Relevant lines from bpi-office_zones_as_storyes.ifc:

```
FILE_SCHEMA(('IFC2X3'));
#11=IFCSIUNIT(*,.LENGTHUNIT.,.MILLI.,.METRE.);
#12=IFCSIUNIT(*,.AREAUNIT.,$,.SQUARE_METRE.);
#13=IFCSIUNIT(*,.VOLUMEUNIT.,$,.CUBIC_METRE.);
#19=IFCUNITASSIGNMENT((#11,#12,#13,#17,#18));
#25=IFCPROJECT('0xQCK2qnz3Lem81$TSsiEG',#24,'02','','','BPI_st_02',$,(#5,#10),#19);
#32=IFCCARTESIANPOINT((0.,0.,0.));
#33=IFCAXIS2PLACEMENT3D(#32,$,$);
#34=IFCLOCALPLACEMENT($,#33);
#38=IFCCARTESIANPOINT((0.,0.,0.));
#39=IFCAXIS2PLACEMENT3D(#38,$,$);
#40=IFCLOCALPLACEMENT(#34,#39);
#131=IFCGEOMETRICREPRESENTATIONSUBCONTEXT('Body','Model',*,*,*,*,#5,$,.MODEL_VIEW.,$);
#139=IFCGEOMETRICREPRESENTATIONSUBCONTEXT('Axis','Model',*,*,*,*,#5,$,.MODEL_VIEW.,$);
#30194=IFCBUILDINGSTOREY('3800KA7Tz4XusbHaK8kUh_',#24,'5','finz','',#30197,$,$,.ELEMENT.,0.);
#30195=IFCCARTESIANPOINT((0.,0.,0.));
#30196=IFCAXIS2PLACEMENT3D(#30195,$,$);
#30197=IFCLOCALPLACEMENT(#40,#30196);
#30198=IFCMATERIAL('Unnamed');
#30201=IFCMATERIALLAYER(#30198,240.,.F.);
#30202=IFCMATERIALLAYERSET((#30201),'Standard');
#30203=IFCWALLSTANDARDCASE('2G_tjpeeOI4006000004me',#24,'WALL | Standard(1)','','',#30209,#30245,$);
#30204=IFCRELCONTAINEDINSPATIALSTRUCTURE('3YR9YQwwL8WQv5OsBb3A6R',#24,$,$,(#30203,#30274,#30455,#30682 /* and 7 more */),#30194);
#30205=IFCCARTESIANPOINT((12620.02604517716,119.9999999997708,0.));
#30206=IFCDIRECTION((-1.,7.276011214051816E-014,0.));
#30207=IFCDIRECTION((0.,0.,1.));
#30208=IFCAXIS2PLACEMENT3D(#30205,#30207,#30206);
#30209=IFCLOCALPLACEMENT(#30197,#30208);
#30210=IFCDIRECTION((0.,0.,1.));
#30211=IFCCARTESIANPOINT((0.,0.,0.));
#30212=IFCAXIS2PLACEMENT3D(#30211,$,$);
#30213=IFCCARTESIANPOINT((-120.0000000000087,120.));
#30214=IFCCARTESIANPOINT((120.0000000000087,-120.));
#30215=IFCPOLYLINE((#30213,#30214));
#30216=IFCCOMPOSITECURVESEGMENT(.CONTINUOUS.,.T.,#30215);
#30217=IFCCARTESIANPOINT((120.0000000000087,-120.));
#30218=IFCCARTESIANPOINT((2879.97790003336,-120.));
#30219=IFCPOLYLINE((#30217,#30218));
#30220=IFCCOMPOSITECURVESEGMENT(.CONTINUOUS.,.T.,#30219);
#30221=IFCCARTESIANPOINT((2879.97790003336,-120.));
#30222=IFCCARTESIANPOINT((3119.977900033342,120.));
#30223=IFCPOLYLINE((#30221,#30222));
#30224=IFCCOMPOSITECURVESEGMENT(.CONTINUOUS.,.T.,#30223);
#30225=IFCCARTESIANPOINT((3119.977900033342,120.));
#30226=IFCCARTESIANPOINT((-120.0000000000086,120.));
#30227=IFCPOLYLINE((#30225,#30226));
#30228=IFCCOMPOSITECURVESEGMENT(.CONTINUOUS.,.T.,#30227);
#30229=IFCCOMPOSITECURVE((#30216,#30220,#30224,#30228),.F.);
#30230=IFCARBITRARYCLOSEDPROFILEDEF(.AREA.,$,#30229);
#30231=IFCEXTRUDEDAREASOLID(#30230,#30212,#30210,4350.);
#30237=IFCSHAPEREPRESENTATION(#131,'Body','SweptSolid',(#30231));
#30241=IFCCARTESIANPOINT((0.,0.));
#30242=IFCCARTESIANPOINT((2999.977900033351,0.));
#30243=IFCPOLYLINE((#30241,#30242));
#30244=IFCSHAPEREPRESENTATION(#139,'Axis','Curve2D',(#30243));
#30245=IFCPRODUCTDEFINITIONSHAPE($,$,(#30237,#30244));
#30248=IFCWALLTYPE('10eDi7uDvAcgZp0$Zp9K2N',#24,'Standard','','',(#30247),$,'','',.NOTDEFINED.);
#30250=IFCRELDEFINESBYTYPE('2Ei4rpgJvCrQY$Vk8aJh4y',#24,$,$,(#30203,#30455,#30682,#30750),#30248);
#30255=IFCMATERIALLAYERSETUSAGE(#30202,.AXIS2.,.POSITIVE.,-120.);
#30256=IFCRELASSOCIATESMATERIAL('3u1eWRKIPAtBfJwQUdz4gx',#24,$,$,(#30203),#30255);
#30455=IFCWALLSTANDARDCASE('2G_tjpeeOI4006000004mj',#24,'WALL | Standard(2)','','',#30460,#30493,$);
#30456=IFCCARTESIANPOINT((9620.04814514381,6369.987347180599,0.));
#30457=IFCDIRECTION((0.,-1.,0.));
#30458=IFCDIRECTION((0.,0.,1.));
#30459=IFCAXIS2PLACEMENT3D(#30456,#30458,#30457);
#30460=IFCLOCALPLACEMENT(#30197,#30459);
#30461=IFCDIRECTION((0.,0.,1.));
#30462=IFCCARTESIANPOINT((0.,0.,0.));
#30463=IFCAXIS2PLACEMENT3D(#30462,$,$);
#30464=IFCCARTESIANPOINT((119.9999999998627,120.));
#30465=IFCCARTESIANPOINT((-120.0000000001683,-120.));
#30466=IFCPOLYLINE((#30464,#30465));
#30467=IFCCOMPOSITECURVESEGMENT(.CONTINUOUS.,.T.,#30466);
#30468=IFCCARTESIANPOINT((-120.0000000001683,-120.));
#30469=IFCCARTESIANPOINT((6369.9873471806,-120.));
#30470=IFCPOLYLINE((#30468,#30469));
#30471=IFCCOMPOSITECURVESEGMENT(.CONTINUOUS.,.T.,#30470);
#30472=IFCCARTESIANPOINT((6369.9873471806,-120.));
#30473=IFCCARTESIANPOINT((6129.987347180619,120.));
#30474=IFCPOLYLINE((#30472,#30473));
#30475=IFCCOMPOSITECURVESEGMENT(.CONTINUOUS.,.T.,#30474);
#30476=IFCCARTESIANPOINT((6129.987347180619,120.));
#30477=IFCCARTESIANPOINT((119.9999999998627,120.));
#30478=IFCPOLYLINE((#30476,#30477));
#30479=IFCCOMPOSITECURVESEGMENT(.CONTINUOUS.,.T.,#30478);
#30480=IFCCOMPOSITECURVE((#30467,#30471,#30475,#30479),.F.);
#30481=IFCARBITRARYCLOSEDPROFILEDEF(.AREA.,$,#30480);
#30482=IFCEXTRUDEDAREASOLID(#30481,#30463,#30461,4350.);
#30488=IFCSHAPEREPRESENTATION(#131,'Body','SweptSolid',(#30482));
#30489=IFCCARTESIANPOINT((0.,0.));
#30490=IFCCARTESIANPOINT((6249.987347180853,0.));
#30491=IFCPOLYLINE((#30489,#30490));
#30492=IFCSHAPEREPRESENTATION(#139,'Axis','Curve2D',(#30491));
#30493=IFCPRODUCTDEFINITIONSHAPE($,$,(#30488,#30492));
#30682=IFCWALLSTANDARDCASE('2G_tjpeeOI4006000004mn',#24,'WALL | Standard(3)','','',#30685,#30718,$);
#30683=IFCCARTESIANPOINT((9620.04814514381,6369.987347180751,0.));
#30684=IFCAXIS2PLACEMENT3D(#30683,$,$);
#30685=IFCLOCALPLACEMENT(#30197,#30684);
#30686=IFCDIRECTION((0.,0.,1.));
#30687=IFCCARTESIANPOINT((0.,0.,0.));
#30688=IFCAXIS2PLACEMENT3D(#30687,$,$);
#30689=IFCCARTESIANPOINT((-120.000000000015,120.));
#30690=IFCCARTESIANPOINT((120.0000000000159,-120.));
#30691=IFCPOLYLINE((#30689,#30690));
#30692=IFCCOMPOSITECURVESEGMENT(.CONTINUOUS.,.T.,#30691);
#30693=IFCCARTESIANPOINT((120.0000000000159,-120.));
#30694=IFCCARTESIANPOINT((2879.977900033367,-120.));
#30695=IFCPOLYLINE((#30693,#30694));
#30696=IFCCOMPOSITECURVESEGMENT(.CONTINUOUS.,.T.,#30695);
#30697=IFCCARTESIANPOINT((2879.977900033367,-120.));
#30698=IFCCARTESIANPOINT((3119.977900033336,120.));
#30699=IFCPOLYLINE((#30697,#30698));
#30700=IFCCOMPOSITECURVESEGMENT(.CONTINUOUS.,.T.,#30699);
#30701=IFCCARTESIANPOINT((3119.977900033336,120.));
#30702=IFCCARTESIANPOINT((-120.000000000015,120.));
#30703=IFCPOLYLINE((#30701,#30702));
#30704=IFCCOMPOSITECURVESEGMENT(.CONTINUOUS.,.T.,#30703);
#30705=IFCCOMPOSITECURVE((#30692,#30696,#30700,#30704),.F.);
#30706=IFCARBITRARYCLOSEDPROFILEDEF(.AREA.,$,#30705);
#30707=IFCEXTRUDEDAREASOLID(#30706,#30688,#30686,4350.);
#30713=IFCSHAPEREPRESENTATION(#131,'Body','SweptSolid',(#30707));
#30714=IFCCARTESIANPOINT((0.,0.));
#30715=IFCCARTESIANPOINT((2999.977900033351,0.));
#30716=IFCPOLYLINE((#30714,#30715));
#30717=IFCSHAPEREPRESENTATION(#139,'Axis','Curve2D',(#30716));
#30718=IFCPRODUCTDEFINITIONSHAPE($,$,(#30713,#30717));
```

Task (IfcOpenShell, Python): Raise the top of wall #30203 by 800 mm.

```python
import ifcopenshell
import ifcopenshell.geom
import ifcopenshell.util.representation
import ifcopenshell.util.shape
import ifcopenshell.util.unit

model = ifcopenshell.open("bpi-office_zones_as_storyes.ifc")
unit_scale = ifcopenshell.util.unit.calculate_unit_scale(model)
settings = ifcopenshell.geom.settings()


def volume(element):
    """Net volume in cubic metres, openings subtracted."""
    shape = ifcopenshell.geom.create_shape(settings, element)
    return ifcopenshell.util.shape.get_volume(shape.geometry)


wall = model.by_guid("2G_tjpeeOI4006000004me")
before = volume(wall)

body = ifcopenshell.util.representation.get_representation(wall, "Model", "Body")
solid = body.Items[0]
old_height = solid.Depth
solid.Depth += 0.8 / unit_scale
after = volume(wall)

print(f"height {old_height:g} -> {solid.Depth:g}, volume {before:.3f} -> {after:.3f} m3")

model.write("bpi-office_zones_as_storyes-out.ifc")
```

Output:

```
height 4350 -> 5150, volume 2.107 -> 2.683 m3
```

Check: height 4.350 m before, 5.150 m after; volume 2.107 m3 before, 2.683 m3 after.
